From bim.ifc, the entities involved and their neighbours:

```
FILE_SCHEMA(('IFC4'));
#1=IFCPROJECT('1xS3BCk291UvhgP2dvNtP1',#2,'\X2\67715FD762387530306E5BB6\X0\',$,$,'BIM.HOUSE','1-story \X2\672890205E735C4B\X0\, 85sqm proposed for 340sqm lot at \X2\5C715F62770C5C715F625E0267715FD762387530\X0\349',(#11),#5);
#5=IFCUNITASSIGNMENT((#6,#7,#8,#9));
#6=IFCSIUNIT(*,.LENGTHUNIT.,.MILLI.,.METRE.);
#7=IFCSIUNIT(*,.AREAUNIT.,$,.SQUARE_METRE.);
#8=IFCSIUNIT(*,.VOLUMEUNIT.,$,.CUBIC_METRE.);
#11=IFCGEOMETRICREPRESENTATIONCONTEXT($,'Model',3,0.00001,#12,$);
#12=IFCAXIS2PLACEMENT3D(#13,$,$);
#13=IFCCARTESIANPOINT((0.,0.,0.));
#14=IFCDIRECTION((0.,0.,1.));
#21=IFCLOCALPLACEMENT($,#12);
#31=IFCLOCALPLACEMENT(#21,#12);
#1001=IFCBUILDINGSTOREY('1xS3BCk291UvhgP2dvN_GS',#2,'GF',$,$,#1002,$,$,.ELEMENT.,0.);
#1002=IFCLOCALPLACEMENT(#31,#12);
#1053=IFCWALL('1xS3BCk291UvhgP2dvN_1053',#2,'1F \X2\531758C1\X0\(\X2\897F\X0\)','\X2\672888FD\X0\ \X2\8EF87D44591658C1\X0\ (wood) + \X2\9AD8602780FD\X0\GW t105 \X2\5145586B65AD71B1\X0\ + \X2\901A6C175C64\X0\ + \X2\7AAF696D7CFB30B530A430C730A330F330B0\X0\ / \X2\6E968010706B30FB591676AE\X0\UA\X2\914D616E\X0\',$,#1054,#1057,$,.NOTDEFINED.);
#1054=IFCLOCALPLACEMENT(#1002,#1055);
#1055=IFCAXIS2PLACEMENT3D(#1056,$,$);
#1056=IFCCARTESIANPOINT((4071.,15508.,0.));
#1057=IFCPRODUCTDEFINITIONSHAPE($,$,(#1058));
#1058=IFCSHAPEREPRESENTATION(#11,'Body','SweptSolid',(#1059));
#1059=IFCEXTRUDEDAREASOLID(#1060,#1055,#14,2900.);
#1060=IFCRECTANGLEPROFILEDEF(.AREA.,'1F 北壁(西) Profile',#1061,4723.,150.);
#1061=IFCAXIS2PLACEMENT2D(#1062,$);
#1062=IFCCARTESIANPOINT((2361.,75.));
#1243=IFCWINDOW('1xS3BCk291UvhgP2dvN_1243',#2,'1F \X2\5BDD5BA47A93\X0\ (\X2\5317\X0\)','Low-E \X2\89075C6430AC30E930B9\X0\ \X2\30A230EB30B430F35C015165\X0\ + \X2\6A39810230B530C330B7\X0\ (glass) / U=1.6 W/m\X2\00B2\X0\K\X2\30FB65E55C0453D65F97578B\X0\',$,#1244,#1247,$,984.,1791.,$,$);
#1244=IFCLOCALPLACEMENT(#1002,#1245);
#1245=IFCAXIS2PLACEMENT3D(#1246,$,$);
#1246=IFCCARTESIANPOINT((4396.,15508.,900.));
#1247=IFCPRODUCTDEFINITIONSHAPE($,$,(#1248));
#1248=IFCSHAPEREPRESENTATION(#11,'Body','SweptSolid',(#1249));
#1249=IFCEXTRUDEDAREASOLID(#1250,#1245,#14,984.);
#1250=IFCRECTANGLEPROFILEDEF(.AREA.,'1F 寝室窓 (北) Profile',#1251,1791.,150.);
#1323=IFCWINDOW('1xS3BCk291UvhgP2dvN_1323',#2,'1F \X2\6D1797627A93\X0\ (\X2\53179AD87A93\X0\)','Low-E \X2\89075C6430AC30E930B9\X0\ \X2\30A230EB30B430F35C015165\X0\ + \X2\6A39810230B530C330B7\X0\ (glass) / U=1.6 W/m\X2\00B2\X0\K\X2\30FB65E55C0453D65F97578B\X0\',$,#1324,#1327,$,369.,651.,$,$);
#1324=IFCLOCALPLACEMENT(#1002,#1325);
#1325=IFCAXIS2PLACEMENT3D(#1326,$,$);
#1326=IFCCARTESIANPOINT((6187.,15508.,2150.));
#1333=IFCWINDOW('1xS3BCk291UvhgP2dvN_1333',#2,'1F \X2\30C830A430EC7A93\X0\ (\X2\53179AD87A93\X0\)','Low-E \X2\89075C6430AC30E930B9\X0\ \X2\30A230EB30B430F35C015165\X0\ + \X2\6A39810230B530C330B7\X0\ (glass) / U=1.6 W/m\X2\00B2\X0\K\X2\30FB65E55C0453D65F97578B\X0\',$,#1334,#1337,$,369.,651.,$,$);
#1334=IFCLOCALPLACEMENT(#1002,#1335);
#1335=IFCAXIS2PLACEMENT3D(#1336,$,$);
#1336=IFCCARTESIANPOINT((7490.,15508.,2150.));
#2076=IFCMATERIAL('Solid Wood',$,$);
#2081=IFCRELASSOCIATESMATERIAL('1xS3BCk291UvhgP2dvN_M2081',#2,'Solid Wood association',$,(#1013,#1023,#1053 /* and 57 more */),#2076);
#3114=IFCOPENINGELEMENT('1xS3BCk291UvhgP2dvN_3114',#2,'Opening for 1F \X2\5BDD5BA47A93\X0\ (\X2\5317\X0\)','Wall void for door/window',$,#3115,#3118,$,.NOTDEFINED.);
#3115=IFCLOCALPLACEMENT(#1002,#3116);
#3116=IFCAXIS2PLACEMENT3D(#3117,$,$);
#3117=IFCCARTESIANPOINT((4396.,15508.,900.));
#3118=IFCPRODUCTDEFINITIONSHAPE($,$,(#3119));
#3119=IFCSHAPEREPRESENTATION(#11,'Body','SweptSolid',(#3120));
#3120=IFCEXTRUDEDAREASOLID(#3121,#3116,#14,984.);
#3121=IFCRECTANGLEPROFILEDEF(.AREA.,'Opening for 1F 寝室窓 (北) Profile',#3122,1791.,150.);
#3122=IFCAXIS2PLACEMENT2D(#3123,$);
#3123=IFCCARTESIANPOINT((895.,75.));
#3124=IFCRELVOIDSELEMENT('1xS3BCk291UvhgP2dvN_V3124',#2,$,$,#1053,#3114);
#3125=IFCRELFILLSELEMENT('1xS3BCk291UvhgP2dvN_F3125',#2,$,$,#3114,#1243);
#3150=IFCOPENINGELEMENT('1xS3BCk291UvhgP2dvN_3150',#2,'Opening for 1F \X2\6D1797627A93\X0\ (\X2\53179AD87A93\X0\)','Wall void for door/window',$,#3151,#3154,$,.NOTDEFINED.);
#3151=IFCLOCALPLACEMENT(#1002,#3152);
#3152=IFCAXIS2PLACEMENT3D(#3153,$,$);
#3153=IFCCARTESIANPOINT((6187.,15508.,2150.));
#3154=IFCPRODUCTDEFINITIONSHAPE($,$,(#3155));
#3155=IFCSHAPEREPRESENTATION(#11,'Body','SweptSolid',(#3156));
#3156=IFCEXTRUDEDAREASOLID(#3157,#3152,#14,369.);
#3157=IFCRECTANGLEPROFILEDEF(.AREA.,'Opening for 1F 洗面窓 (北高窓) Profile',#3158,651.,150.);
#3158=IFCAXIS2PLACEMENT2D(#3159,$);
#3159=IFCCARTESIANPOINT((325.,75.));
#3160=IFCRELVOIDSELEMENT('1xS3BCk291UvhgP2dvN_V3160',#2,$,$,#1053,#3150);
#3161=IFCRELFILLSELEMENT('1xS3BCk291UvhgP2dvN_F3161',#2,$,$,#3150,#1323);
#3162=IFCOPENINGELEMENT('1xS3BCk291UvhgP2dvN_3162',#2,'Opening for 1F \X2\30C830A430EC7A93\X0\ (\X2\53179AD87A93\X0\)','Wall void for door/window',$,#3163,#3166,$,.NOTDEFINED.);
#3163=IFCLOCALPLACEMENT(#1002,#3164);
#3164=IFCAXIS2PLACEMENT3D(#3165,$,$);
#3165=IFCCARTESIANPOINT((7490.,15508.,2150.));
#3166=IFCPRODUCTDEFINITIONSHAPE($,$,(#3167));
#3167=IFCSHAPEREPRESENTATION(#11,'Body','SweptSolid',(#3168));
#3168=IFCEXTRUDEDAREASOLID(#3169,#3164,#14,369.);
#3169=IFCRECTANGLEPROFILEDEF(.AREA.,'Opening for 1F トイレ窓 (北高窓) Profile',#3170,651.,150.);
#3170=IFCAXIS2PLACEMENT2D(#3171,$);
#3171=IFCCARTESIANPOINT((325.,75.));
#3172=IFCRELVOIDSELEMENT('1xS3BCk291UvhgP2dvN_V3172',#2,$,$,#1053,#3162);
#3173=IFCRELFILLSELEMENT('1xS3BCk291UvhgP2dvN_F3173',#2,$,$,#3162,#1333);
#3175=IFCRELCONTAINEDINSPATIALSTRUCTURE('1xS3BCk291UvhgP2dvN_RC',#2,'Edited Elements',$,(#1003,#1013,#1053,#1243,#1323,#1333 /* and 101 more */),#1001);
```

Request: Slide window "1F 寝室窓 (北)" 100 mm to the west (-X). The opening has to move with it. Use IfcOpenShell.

```python
import ifcopenshell
import ifcopenshell.api.geometry
import ifcopenshell.util.placement

model = ifcopenshell.open("bim.ifc")

window = model.by_guid("1xS3BCk291UvhgP2dvN_1243")
opening = window.FillsVoids[0].RelatingOpeningElement
wall = opening.VoidsElements[0].RelatingBuildingElement

wall_matrix = ifcopenshell.util.placement.get_local_placement(wall.ObjectPlacement)
shift = wall_matrix[:3, 0] * -100.0
before = ifcopenshell.util.placement.get_local_placement(window.ObjectPlacement)[:3, 3].copy()

# The window is not placed relative to its opening, so move both.
for product in (opening, window):
    matrix = ifcopenshell.util.placement.get_local_placement(product.ObjectPlacement)
    matrix[:3, 3] += shift
    ifcopenshell.api.geometry.edit_object_placement(model, product=product, matrix=matrix, is_si=False)

after = ifcopenshell.util.placement.get_local_placement(window.ObjectPlacement)[:3, 3]
print("window moved by", (after - before).round(3) + 0.0)

model.write("bim_edited.ifc")
```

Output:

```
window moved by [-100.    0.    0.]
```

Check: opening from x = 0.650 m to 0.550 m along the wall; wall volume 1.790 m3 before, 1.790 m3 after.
